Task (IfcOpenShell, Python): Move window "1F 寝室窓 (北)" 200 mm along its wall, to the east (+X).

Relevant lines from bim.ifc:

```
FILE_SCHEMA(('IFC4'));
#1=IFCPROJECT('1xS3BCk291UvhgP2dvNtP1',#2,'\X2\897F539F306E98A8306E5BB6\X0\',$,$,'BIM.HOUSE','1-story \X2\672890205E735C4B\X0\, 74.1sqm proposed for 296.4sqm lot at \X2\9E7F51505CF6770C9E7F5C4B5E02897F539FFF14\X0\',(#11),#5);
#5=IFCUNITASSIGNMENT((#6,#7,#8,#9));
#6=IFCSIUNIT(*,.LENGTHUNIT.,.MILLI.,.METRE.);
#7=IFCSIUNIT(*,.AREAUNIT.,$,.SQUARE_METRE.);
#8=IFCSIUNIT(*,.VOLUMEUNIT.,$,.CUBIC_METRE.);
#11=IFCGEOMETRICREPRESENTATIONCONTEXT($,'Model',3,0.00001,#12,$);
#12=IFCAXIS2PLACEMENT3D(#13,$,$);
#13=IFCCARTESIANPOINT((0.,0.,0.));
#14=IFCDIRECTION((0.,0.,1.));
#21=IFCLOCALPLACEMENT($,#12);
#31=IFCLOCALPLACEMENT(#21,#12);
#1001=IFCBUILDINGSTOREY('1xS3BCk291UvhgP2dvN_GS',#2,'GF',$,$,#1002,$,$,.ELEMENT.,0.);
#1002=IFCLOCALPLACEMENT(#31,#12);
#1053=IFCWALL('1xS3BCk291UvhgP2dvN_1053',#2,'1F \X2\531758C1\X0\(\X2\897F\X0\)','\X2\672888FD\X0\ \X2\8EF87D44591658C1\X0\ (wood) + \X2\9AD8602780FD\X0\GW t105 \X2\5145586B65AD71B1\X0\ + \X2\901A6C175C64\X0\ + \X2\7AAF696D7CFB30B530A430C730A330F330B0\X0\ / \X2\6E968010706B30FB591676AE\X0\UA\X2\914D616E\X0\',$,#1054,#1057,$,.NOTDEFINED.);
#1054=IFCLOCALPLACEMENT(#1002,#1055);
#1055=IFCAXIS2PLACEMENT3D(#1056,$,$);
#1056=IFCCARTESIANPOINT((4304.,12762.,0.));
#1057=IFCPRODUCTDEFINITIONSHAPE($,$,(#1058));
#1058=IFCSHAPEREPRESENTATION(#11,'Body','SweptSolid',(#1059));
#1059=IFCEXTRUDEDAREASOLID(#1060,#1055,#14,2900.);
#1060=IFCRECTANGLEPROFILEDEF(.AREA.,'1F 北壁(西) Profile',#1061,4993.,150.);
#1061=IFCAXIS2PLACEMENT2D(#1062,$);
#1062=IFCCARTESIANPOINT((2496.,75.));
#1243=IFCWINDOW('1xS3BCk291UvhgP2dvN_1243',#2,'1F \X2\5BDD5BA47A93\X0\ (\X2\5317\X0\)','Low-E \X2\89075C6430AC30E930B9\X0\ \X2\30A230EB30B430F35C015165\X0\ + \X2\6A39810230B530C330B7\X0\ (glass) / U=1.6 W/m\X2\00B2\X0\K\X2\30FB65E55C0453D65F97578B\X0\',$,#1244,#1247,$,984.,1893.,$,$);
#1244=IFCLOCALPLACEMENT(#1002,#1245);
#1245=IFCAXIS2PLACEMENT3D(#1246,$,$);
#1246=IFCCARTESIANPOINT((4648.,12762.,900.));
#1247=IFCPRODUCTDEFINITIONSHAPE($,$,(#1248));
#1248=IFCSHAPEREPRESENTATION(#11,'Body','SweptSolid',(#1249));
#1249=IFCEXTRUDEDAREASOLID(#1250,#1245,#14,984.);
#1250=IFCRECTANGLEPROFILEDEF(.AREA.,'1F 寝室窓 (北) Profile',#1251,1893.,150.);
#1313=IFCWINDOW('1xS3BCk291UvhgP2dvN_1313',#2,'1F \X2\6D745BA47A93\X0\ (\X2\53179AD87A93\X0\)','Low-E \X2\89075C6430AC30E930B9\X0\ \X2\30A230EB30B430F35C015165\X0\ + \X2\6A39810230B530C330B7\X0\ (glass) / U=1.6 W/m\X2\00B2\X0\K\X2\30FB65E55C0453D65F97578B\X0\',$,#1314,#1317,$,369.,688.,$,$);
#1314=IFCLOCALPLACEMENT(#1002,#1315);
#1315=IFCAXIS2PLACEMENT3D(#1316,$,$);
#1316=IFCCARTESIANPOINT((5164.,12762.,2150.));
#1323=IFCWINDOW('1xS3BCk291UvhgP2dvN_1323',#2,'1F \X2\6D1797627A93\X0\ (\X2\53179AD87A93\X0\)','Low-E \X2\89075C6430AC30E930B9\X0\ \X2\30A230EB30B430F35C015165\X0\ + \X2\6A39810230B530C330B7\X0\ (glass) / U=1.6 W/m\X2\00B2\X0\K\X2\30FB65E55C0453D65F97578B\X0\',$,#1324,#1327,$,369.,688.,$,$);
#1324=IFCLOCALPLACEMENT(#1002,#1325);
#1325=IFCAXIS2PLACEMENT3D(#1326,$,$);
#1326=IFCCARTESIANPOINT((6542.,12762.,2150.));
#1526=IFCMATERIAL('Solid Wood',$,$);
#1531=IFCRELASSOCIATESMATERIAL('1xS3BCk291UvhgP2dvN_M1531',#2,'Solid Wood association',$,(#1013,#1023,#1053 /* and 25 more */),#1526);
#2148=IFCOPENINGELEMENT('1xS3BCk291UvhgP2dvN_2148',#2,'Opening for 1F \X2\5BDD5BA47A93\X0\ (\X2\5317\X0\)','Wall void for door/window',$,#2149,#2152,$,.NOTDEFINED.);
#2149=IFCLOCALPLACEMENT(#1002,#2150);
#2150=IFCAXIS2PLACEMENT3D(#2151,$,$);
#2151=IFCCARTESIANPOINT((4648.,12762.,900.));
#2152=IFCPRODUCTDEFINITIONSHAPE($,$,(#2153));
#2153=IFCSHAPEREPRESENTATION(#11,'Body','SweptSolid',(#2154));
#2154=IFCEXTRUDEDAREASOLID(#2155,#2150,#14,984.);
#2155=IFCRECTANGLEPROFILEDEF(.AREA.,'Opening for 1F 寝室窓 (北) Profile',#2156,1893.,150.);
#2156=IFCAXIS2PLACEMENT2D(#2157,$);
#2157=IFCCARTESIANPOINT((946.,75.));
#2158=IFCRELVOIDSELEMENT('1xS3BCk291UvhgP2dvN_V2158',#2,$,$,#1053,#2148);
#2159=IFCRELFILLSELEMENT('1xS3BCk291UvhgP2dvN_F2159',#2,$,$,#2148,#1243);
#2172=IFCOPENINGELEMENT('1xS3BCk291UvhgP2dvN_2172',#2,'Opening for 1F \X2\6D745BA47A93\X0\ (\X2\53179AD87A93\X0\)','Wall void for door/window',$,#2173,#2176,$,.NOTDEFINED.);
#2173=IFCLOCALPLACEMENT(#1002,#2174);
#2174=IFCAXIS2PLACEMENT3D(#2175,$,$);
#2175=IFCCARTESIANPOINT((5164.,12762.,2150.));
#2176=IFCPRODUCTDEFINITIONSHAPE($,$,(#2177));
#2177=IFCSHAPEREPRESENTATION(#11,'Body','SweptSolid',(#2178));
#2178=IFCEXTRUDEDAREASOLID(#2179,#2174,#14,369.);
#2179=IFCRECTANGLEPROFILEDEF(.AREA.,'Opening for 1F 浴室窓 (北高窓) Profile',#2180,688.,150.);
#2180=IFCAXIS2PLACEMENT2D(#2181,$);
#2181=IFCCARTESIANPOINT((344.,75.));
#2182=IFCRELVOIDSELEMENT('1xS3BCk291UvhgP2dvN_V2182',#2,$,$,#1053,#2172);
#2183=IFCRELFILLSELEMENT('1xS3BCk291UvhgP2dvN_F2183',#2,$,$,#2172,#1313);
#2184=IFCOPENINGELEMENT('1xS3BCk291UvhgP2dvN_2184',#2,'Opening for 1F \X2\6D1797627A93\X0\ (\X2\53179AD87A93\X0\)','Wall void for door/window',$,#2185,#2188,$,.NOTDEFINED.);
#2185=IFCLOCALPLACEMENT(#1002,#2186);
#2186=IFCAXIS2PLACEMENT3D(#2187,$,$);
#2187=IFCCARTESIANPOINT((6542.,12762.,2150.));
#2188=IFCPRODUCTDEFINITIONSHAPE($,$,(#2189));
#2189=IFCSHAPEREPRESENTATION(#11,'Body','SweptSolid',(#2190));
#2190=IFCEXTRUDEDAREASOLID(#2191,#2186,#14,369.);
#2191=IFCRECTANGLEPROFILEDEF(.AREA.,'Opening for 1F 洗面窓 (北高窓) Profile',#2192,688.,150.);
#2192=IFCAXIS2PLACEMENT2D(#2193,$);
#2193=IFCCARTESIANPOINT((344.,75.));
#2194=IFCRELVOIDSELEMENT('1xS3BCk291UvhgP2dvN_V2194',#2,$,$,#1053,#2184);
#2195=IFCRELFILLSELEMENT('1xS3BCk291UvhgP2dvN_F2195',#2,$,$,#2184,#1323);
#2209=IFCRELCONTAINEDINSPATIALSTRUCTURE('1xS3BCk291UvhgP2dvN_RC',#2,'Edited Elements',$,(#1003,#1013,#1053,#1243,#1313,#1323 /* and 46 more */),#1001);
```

```python
import ifcopenshell
import ifcopenshell.api.geometry
import ifcopenshell.util.placement

model = ifcopenshell.open("bim.ifc")

window = model.by_guid("1xS3BCk291UvhgP2dvN_1243")
opening = window.FillsVoids[0].RelatingOpeningElement
wall = opening.VoidsElements[0].RelatingBuildingElement

wall_matrix = ifcopenshell.util.placement.get_local_placement(wall.ObjectPlacement)
shift = wall_matrix[:3, 0] * 200.0
before = ifcopenshell.util.placement.get_local_placement(window.ObjectPlacement)[:3, 3].copy()

# The window is not placed relative to its opening, so move both.
for product in (opening, window):
    matrix = ifcopenshell.util.placement.get_local_placement(product.ObjectPlacement)
    matrix[:3, 3] += shift
    ifcopenshell.api.geometry.edit_object_placement(model, product=product, matrix=matrix, is_si=False)

after = ifcopenshell.util.placement.get_local_placement(window.ObjectPlacement)[:3, 3]
print("window moved by", (after - before).round(3) + 0.0)

model.write("bim_edited.ifc")
```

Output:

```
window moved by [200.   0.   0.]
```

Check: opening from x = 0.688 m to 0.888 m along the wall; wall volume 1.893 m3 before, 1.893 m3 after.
